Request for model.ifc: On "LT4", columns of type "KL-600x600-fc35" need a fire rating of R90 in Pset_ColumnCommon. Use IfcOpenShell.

First a look at what the model holds.

```python
import ifcopenshell
import ifcopenshell.util.element

model = ifcopenshell.open("model.ifc")
print(model.schema)
storey = next(s for s in model.by_type("IfcBuildingStorey") if s.Name == "LT4")
columns = [e for e in ifcopenshell.util.element.get_decomposition(storey) if e.is_a("IfcColumn")]
seen = {}
for e in columns:
    element_type = ifcopenshell.util.element.get_type(e)
    key = (element_type.Name if element_type != e and element_type else None, ifcopenshell.util.element.get_pset(e, "Pset_ColumnCommon", "FireRating"))
    seen[key] = seen.get(key, 0) + 1
for (name, value), count in sorted(seen.items(), key=str):
    print(count, "x", name, "|", value)
```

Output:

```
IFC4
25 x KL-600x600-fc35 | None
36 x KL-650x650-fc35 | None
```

```python
import ifcopenshell
import ifcopenshell.api.pset
import ifcopenshell.util.element

model = ifcopenshell.open("model.ifc")

storey = next(s for s in model.by_type("IfcBuildingStorey") if s.Name == "LT4")
columns = [e for e in ifcopenshell.util.element.get_decomposition(storey) if e.is_a("IfcColumn")]

count = 0
for e in columns:
    element_type = ifcopenshell.util.element.get_type(e)
    if element_type in (None, e) or element_type.Name != "KL-600x600-fc35":
        continue
    # add_pset returns the element's existing set when there is one.
    pset = ifcopenshell.api.pset.add_pset(model, product=e, name="Pset_ColumnCommon")
    ifcopenshell.api.pset.edit_pset(model, pset=pset, properties={"FireRating": "R90"})
    count += 1

print(count, "columns updated")

model.write("model_updated.ifc")
```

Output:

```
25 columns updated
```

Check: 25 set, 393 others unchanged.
